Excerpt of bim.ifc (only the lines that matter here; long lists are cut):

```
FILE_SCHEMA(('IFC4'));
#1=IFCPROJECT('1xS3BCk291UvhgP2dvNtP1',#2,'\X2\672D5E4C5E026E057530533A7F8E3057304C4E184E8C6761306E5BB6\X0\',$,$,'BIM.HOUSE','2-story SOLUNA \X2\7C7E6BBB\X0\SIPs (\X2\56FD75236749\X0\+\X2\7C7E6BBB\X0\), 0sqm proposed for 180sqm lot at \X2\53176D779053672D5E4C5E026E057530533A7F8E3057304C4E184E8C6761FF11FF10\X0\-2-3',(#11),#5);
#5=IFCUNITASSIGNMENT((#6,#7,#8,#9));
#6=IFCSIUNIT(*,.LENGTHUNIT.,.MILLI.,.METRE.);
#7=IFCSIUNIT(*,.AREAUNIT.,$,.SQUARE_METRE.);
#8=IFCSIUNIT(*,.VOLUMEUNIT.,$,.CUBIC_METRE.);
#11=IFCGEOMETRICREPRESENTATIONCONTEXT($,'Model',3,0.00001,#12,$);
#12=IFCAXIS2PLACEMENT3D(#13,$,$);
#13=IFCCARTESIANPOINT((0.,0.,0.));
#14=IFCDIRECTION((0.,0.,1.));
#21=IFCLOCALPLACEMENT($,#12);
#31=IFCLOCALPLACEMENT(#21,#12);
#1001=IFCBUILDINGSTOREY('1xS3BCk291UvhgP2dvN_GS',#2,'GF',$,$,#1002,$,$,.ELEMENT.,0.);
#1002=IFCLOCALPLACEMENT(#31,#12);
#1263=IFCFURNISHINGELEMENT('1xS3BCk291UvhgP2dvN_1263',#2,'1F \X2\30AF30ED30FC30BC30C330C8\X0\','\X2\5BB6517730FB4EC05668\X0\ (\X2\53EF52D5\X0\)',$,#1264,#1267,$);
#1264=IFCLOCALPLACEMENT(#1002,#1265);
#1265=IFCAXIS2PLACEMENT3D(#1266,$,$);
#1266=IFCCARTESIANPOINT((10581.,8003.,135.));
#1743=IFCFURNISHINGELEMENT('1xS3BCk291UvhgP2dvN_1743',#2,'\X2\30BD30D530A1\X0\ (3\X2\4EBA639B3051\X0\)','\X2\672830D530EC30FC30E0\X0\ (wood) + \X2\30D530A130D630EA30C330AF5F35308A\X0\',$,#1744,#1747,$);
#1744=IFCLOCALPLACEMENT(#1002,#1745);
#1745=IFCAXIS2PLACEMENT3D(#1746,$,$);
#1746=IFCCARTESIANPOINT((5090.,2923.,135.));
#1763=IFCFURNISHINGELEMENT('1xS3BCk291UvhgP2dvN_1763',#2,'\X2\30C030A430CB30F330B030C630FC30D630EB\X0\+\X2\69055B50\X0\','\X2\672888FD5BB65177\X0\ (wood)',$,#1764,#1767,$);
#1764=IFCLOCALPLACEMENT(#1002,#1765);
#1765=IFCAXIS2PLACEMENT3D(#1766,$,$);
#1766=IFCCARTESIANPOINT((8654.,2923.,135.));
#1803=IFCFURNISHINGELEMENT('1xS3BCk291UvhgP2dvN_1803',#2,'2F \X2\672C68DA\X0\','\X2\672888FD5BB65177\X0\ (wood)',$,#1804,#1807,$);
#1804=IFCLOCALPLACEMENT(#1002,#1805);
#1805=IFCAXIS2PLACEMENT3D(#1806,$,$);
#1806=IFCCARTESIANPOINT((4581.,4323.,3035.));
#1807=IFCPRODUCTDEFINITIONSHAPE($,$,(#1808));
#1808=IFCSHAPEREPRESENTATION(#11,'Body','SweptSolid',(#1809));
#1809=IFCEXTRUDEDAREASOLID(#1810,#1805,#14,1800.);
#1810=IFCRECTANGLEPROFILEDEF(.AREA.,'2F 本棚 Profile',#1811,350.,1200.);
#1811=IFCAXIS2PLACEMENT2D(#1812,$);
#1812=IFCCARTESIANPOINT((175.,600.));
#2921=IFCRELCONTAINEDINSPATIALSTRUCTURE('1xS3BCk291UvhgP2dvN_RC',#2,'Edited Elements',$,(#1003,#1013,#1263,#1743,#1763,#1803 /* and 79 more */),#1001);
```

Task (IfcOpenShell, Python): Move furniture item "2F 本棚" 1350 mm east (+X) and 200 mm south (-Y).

```python
import ifcopenshell
import ifcopenshell.api.geometry
import ifcopenshell.util.placement
import ifcopenshell.util.unit

model = ifcopenshell.open("bim.ifc")
unit_scale = ifcopenshell.util.unit.calculate_unit_scale(model)

item = model.by_guid("1xS3BCk291UvhgP2dvN_1803")
matrix = ifcopenshell.util.placement.get_local_placement(item.ObjectPlacement)
matrix[0, 3] += 1.35 / unit_scale
matrix[1, 3] -= 0.2 / unit_scale
ifcopenshell.api.geometry.edit_object_placement(model, product=item, matrix=matrix, is_si=False)

print(ifcopenshell.util.placement.get_local_placement(item.ObjectPlacement).round(3) + 0.0)

model.write("bim_v2.ifc")
```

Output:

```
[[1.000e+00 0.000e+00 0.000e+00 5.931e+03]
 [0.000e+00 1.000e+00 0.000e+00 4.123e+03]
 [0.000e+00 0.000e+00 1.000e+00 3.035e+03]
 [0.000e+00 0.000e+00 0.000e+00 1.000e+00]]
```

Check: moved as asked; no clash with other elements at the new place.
